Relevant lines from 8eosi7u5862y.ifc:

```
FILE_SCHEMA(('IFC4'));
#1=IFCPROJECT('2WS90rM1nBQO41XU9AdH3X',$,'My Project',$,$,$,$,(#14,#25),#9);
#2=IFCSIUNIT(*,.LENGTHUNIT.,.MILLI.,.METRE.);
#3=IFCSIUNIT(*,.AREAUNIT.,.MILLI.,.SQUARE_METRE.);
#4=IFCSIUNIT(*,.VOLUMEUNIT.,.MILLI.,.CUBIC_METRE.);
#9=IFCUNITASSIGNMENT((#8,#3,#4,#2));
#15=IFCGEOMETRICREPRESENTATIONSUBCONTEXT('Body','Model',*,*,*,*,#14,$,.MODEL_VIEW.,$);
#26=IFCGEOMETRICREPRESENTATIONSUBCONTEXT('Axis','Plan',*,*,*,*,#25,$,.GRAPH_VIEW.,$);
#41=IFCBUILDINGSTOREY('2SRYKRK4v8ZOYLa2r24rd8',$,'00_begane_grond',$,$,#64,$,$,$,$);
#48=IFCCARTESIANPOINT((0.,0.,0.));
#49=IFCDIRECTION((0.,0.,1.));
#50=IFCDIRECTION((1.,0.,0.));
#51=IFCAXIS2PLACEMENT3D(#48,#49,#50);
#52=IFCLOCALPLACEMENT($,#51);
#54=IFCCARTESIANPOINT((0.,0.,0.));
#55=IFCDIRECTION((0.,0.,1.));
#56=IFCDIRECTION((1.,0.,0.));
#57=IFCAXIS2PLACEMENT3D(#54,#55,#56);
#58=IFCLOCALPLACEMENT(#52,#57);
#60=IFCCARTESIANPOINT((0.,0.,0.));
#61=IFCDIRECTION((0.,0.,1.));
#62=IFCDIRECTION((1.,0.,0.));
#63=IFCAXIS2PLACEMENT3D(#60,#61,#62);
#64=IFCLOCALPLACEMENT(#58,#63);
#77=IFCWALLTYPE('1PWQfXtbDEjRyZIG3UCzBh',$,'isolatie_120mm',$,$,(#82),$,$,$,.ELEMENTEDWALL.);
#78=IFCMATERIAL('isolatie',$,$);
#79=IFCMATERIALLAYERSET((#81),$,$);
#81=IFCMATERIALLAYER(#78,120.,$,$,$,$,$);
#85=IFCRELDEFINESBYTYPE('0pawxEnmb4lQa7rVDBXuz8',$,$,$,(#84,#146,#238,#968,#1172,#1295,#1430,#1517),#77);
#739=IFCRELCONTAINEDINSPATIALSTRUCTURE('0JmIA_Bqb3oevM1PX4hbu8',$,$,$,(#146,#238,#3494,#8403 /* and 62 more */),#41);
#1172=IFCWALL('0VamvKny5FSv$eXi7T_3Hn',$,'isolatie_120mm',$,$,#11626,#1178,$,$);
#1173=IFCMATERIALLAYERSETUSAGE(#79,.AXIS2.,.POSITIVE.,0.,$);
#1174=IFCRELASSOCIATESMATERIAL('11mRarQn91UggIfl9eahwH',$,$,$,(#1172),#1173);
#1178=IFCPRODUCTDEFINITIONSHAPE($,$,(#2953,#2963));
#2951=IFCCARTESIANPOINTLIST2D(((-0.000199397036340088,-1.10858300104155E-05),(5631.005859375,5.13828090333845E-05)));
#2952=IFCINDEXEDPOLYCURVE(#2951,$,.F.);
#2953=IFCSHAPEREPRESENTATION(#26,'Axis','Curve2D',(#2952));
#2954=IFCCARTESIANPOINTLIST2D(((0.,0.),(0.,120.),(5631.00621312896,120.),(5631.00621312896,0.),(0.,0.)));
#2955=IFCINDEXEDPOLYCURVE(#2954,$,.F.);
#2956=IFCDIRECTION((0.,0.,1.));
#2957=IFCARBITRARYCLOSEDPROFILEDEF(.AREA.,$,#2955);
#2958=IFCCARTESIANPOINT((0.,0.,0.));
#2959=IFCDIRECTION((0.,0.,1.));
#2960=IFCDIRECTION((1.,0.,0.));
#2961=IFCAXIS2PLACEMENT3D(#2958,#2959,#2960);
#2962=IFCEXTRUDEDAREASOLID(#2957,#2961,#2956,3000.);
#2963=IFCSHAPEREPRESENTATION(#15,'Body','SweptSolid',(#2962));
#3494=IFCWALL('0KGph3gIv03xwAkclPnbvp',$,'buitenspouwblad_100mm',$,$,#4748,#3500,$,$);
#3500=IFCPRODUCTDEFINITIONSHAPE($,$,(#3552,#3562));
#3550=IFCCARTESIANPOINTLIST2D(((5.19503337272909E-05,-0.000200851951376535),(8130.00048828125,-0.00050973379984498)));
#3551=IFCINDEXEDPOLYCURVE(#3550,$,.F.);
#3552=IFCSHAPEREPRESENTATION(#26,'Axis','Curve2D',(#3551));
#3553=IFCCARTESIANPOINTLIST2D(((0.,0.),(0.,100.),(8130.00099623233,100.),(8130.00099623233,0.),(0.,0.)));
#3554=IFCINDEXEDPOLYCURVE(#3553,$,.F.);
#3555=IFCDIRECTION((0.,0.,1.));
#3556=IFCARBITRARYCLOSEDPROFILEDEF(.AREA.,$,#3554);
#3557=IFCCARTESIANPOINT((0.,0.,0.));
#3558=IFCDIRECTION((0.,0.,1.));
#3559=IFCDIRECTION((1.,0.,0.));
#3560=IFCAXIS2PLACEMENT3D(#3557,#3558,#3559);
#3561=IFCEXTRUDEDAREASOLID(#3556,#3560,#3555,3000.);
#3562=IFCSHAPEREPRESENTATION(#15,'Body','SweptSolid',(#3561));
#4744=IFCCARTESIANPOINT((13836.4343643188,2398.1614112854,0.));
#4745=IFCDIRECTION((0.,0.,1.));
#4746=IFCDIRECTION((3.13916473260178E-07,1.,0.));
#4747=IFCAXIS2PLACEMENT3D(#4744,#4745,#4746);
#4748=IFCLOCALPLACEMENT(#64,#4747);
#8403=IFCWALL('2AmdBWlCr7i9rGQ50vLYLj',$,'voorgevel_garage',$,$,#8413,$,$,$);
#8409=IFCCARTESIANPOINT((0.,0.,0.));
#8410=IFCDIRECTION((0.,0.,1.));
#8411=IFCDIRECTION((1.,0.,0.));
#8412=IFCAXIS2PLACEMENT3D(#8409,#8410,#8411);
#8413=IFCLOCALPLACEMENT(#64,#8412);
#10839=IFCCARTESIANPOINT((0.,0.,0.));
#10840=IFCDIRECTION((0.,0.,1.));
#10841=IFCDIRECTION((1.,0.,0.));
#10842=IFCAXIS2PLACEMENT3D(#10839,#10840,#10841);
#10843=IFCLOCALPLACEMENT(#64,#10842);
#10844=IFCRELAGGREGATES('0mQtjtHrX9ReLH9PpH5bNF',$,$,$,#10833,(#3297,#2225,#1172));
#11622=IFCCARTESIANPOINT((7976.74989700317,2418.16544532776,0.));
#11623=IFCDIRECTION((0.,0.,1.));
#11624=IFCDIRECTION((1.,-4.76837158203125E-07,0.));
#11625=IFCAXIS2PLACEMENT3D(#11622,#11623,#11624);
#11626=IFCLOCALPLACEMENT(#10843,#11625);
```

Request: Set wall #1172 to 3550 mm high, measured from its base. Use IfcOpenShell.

```python
import ifcopenshell
import ifcopenshell.geom
import ifcopenshell.util.representation
import ifcopenshell.util.shape

model = ifcopenshell.open("8eosi7u5862y.ifc")
settings = ifcopenshell.geom.settings()


def volume(element):
    """Net volume in cubic metres, openings subtracted."""
    shape = ifcopenshell.geom.create_shape(settings, element)
    return ifcopenshell.util.shape.get_volume(shape.geometry)


wall = model.by_guid("0VamvKny5FSv$eXi7T_3Hn")
before = volume(wall)

body = ifcopenshell.util.representation.get_representation(wall, "Model", "Body")
solid = body.Items[0]
old_height = solid.Depth
solid.Depth = 3550.0
after = volume(wall)

print(f"height {old_height:g} -> {solid.Depth:g}, volume {before:.3f} -> {after:.3f} m3")

model.write("8eosi7u5862y_updated.ifc")
```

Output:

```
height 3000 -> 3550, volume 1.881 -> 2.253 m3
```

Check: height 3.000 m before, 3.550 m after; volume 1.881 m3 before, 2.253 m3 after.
